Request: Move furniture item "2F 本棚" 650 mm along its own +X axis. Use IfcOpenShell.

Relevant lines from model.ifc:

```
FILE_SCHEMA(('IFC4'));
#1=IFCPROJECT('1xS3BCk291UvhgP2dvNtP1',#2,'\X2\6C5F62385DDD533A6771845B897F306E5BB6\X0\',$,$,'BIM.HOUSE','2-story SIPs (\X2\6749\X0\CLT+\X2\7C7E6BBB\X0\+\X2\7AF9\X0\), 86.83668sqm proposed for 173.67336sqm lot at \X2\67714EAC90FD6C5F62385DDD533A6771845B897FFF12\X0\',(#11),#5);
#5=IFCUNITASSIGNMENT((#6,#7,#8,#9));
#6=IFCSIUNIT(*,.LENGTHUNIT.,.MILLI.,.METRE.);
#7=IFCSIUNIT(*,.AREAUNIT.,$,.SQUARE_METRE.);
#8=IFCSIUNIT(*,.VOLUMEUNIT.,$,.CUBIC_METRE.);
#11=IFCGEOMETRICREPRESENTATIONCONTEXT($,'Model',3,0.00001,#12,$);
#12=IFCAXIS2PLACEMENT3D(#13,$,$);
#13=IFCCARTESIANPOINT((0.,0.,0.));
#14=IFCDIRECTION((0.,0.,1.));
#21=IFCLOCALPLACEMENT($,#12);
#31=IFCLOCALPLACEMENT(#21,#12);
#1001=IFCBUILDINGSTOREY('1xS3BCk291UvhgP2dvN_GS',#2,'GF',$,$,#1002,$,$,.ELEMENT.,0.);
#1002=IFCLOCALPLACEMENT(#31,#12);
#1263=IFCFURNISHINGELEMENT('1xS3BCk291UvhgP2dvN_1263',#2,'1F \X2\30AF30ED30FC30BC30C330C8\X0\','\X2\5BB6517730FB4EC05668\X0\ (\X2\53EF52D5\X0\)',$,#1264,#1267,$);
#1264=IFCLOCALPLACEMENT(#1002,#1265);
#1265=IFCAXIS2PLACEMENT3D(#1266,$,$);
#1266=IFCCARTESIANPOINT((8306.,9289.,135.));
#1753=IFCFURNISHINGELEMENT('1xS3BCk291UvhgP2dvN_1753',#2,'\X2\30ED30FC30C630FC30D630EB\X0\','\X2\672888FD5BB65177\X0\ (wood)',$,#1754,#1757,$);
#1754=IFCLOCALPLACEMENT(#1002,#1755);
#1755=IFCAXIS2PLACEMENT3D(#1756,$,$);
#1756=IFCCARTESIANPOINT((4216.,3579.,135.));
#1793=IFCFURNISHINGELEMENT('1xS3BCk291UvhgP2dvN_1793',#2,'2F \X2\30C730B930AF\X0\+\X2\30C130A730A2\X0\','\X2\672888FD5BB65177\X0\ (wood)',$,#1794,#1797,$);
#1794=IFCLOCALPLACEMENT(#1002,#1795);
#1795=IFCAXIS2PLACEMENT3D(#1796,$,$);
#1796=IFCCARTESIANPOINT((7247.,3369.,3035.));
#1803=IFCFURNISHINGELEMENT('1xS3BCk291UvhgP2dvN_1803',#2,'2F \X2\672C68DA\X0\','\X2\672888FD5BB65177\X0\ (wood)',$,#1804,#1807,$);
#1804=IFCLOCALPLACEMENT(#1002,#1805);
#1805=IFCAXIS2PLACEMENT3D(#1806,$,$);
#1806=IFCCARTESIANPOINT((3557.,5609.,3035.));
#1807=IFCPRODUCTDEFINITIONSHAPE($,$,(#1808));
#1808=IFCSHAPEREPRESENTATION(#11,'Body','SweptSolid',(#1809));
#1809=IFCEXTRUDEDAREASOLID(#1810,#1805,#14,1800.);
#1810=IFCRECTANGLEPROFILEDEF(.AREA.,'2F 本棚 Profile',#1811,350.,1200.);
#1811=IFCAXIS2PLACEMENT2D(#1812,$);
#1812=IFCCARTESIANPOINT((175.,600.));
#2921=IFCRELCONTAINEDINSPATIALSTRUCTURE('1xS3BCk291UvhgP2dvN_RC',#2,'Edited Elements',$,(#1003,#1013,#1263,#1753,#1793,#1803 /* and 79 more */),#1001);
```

```python
import ifcopenshell
import ifcopenshell.api.geometry
import ifcopenshell.util.placement
import ifcopenshell.util.unit

model = ifcopenshell.open("model.ifc")
unit_scale = ifcopenshell.util.unit.calculate_unit_scale(model)

item = model.by_guid("1xS3BCk291UvhgP2dvN_1803")
matrix = ifcopenshell.util.placement.get_local_placement(item.ObjectPlacement)
matrix[:3, 3] += matrix[:3, 0] * 0.65 / unit_scale
ifcopenshell.api.geometry.edit_object_placement(model, product=item, matrix=matrix, is_si=False)

print(ifcopenshell.util.placement.get_local_placement(item.ObjectPlacement).round(3) + 0.0)

model.write("model_edited.ifc")
```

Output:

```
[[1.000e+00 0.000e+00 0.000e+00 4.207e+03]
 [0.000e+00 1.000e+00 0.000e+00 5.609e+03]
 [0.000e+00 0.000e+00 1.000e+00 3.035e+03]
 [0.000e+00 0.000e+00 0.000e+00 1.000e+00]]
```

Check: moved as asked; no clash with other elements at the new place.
